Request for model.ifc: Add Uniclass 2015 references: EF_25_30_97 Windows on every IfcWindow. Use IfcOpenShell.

First a look at what the model holds.

```python
import ifcopenshell

model = ifcopenshell.open("model.ifc")
print(model.schema)
print("classifications:", [c.Name for c in model.by_type("IfcClassification")])
for ifc_class in ("IfcDoor", "IfcRoof", "IfcStair", "IfcWall", "IfcWindow"):
    print(ifc_class, len(model.by_type(ifc_class)))
```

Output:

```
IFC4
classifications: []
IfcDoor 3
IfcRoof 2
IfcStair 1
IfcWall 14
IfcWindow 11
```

```python
import ifcopenshell
import ifcopenshell.api.classification

model = ifcopenshell.open("model.ifc")

system = ifcopenshell.api.classification.add_classification(model, classification="Uniclass 2015")

codes = {
    "IfcWindow": ("EF_25_30_97", "Windows"),
}
for ifc_class, (code, name) in codes.items():
    products = model.by_type(ifc_class)
    ifcopenshell.api.classification.add_reference(
        model, products=products, classification=system, identification=code, name=name
    )
    print(code, len(products))

model.write("model_v2.ifc")
```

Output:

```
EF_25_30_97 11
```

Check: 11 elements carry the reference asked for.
